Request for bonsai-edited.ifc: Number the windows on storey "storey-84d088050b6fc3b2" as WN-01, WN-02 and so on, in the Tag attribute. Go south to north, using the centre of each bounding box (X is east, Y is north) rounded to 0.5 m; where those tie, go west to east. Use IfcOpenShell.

First a look at what the model holds.

```python
import ifcopenshell
import ifcopenshell.util.element
import ifcopenshell.util.placement

model = ifcopenshell.open("bonsai-edited.ifc")
print(model.schema)
storey = next(s for s in model.by_type("IfcBuildingStorey") if s.Name == "storey-84d088050b6fc3b2")
windows = [e for e in ifcopenshell.util.element.get_decomposition(storey) if e.is_a("IfcWindow")]
for e in sorted(windows, key=lambda e: e.id()):
    origin = ifcopenshell.util.placement.get_local_placement(e.ObjectPlacement)[:3, 3]
    print(e.id(), e.Tag, e.Name, origin.round(2) + 0.0, sep=" | ")
```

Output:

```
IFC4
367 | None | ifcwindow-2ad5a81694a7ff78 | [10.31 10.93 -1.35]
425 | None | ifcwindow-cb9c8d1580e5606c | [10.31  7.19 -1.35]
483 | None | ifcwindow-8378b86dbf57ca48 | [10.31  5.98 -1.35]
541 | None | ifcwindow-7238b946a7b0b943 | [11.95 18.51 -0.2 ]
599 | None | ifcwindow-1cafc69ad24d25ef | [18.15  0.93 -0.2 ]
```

```python
import ifcopenshell
import ifcopenshell.geom
import ifcopenshell.util.element
import ifcopenshell.util.shape

model = ifcopenshell.open("bonsai-edited.ifc")
settings = ifcopenshell.geom.settings()
settings.set("use-world-coords", True)


def centre(element):
    shape = ifcopenshell.geom.create_shape(settings, element)
    return ifcopenshell.util.shape.get_bbox_centroid(shape.geometry)


storey = next(s for s in model.by_type("IfcBuildingStorey") if s.Name == "storey-84d088050b6fc3b2")
windows = [e for e in ifcopenshell.util.element.get_decomposition(storey) if e.is_a("IfcWindow")]

# Insertion points can sit at a corner or the storey origin, so sort by the geometry (in metres).
centres = {e: centre(e) for e in windows}
windows.sort(key=lambda e: (round(centres[e][1] / 0.5), centres[e][0]))

for i, e in enumerate(windows, start=1):
    number = f"WN-{i:02d}"
    e.Tag = number
    print(e.id(), number)

model.write("bonsai-edited-out.ifc")
```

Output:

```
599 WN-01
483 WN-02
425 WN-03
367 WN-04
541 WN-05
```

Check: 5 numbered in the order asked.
